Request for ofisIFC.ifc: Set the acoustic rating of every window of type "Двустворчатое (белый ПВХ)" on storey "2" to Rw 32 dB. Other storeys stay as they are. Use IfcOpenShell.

First a look at what the model holds.

```python
import ifcopenshell
import ifcopenshell.util.element

model = ifcopenshell.open("ofisIFC.ifc")
print(model.schema)
storey = next(s for s in model.by_type("IfcBuildingStorey") if s.Name == "2")
windows = [e for e in ifcopenshell.util.element.get_decomposition(storey) if e.is_a("IfcWindow")]
seen = {}
for e in windows:
    element_type = ifcopenshell.util.element.get_type(e)
    key = (element_type.Name if element_type != e and element_type else None, ifcopenshell.util.element.get_pset(e, "Pset_WindowCommon", "AcousticRating"))
    seen[key] = seen.get(key, 0) + 1
for (name, value), count in sorted(seen.items(), key=str):
    print(count, "x", name, "|", value)
```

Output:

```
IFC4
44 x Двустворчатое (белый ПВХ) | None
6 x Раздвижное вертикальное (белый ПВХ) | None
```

```python
import ifcopenshell
import ifcopenshell.api.pset
import ifcopenshell.util.element

model = ifcopenshell.open("ofisIFC.ifc")

storey = next(s for s in model.by_type("IfcBuildingStorey") if s.Name == "2")
windows = [e for e in ifcopenshell.util.element.get_decomposition(storey) if e.is_a("IfcWindow")]

count = 0
for e in windows:
    element_type = ifcopenshell.util.element.get_type(e)
    if element_type in (None, e) or element_type.Name != "Двустворчатое (белый ПВХ)":
        continue
    # add_pset returns the element's existing set when there is one.
    pset = ifcopenshell.api.pset.add_pset(model, product=e, name="Pset_WindowCommon")
    ifcopenshell.api.pset.edit_pset(model, pset=pset, properties={"AcousticRating": "Rw 32 dB"})
    count += 1

print(count, "windows updated")

model.write("ofisIFC_edited.ifc")
```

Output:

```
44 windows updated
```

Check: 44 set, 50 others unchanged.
